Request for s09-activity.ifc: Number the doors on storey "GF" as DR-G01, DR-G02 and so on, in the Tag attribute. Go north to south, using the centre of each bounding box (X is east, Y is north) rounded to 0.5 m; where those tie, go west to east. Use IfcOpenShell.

First a look at what the model holds.

```python
import ifcopenshell
import ifcopenshell.util.element
import ifcopenshell.util.placement

model = ifcopenshell.open("s09-activity.ifc")
print(model.schema)
storey = next(s for s in model.by_type("IfcBuildingStorey") if s.Name == "GF")
doors = [e for e in ifcopenshell.util.element.get_decomposition(storey) if e.is_a("IfcDoor")]
for e in sorted(doors, key=lambda e: e.id()):
    origin = ifcopenshell.util.placement.get_local_placement(e.ObjectPlacement)[:3, 3]
    print(e.id(), e.Tag, e.Name, origin.round(2) + 0.0, sep=" | ")
```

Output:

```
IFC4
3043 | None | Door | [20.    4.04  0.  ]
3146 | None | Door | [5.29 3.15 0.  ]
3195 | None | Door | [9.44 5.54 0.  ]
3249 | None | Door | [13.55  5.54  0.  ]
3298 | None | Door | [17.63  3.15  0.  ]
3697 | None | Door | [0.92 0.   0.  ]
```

```python
import ifcopenshell
import ifcopenshell.geom
import ifcopenshell.util.element
import ifcopenshell.util.shape

model = ifcopenshell.open("s09-activity.ifc")
settings = ifcopenshell.geom.settings()
settings.set("use-world-coords", True)


def centre(element):
    shape = ifcopenshell.geom.create_shape(settings, element)
    return ifcopenshell.util.shape.get_bbox_centroid(shape.geometry)


storey = next(s for s in model.by_type("IfcBuildingStorey") if s.Name == "GF")
doors = [e for e in ifcopenshell.util.element.get_decomposition(storey) if e.is_a("IfcDoor")]

# Insertion points can sit at a corner or the storey origin, so sort by the geometry (in metres).
centres = {e: centre(e) for e in doors}
doors.sort(key=lambda e: (-round(centres[e][1] / 0.5), centres[e][0]))

for i, e in enumerate(doors, start=1):
    number = f"DR-G{i:02d}"
    e.Tag = number
    print(e.id(), number)

model.write("s09-activity_v2.ifc")
```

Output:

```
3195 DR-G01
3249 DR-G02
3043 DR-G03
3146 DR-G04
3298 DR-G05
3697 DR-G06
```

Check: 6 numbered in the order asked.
